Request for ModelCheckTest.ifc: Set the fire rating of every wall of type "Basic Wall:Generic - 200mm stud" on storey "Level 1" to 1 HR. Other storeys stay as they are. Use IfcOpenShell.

First a look at what the model holds.

```python
import ifcopenshell
import ifcopenshell.util.element

model = ifcopenshell.open("ModelCheckTest.ifc")
print(model.schema)
storey = next(s for s in model.by_type("IfcBuildingStorey") if s.Name == "Level 1")
walls = [e for e in ifcopenshell.util.element.get_decomposition(storey) if e.is_a("IfcWall")]
seen = {}
for e in walls:
    element_type = ifcopenshell.util.element.get_type(e)
    key = (element_type.Name if element_type != e and element_type else None, ifcopenshell.util.element.get_pset(e, "Pset_WallCommon", "FireRating"))
    seen[key] = seen.get(key, 0) + 1
for (name, value), count in sorted(seen.items(), key=str):
    print(count, "x", name, "|", value)
```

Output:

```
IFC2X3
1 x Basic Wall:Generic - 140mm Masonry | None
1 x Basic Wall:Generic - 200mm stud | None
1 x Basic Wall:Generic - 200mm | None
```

```python
import ifcopenshell
import ifcopenshell.api.pset
import ifcopenshell.util.element

model = ifcopenshell.open("ModelCheckTest.ifc")

storey = next(s for s in model.by_type("IfcBuildingStorey") if s.Name == "Level 1")
walls = [e for e in ifcopenshell.util.element.get_decomposition(storey) if e.is_a("IfcWall")]

count = 0
for e in walls:
    element_type = ifcopenshell.util.element.get_type(e)
    if element_type in (None, e) or element_type.Name != "Basic Wall:Generic - 200mm stud":
        continue
    # add_pset returns the element's existing set when there is one.
    pset = ifcopenshell.api.pset.add_pset(model, product=e, name="Pset_WallCommon")
    ifcopenshell.api.pset.edit_pset(model, pset=pset, properties={"FireRating": "1 HR"})
    count += 1

print(count, "walls updated")

model.write("ModelCheckTest_rev.ifc")
```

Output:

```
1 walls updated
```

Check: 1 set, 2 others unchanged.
